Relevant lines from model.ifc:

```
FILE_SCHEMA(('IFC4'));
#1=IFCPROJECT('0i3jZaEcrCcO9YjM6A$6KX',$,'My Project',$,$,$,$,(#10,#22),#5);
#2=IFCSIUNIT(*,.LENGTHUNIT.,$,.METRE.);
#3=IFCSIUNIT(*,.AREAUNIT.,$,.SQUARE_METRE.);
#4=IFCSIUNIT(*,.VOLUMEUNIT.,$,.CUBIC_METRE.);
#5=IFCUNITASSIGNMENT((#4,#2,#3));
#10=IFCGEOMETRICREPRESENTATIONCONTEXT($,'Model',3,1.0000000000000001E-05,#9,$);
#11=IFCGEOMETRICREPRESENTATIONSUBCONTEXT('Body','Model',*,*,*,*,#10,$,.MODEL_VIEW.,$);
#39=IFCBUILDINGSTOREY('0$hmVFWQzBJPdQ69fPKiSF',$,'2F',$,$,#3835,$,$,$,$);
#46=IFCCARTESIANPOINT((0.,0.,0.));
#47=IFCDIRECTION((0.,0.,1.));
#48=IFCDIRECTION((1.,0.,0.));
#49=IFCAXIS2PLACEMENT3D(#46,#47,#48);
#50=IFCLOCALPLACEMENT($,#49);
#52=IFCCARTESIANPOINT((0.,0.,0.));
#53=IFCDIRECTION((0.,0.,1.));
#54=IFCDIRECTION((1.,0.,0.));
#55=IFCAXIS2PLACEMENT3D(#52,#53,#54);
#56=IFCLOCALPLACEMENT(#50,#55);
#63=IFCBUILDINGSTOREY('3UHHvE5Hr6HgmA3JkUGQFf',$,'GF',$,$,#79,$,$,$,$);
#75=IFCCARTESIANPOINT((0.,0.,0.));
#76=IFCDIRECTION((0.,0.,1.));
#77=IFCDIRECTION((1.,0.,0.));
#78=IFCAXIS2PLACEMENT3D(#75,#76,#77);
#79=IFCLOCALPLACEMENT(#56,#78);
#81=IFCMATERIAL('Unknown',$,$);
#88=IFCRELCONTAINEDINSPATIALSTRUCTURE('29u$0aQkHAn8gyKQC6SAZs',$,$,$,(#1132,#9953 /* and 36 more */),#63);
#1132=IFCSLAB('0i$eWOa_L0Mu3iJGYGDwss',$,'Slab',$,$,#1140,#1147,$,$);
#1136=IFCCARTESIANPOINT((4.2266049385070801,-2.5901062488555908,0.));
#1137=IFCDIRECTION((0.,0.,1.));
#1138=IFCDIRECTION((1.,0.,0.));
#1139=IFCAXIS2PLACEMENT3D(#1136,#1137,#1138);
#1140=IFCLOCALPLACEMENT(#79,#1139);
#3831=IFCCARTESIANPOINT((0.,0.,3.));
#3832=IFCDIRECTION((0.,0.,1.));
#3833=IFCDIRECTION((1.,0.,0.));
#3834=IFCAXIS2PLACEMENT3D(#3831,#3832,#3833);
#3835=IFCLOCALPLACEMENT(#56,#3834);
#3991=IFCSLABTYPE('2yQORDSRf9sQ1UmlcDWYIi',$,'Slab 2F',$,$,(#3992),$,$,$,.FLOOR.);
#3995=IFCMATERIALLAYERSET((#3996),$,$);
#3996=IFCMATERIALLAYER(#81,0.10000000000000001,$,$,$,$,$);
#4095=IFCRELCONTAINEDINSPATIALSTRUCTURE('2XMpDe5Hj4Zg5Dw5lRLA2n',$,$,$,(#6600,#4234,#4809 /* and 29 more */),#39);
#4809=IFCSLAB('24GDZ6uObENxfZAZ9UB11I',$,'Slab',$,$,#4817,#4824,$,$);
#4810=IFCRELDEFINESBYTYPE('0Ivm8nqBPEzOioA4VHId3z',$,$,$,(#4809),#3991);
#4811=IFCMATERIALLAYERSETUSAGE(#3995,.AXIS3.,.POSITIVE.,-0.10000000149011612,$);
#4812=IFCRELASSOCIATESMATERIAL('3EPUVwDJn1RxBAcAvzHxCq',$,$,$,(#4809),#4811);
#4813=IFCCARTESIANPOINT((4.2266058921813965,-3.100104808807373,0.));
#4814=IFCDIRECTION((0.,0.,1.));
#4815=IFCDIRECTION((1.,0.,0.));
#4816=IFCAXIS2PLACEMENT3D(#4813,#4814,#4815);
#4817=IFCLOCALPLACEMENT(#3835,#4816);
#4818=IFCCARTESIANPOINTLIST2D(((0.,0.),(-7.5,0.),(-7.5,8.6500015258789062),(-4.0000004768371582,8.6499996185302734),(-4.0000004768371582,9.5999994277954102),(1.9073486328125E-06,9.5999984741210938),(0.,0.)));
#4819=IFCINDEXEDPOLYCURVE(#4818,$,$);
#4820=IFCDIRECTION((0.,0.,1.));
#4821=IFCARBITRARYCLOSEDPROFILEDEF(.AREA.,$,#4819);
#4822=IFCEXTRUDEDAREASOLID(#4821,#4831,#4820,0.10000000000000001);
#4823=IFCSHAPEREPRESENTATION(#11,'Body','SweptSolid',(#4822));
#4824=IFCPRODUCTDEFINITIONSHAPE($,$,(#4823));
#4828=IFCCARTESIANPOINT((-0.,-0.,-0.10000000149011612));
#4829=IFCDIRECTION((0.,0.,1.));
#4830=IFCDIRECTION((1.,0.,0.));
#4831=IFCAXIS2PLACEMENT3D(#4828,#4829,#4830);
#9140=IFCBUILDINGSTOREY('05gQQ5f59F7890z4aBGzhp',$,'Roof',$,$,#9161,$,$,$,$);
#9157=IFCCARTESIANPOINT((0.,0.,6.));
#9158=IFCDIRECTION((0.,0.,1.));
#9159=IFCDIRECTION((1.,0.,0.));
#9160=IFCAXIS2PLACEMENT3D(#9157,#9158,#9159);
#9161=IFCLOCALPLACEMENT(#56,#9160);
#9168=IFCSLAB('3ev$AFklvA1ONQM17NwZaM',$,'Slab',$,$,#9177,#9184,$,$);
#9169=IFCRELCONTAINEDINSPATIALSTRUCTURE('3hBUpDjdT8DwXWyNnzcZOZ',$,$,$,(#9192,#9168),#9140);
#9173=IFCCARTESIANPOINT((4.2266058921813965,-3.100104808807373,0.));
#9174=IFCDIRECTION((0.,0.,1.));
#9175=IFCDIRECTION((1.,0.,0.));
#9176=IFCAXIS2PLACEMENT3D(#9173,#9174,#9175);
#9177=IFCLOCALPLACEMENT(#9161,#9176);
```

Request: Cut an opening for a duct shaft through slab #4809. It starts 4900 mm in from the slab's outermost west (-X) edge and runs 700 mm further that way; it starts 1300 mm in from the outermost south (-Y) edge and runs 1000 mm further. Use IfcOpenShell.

```python
import numpy as np
import ifcopenshell
import ifcopenshell.api.feature
import ifcopenshell.api.geometry
import ifcopenshell.api.root
import ifcopenshell.geom
import ifcopenshell.util.placement
import ifcopenshell.util.representation
import ifcopenshell.util.shape
import ifcopenshell.util.unit

model = ifcopenshell.open("model.ifc")
unit_scale = ifcopenshell.util.unit.calculate_unit_scale(model)
settings = ifcopenshell.geom.settings()


def volume(element):
    """Net volume in cubic metres, openings subtracted."""
    shape = ifcopenshell.geom.create_shape(settings, element)
    return ifcopenshell.util.shape.get_volume(shape.geometry)


slab = model.by_guid("24GDZ6uObENxfZAZ9UB11I")
before = volume(slab)

# Extent in the slab's own axes, in metres. The edges named are its -X and -Y sides.
slab_shape = ifcopenshell.geom.create_shape(settings, slab)
vertices = ifcopenshell.util.shape.get_vertices(slab_shape.geometry)
x_min, y_min, bottom = vertices.min(axis=0)
top = vertices[:, 2].max()

opening = ifcopenshell.api.root.create_entity(model, ifc_class="IfcOpeningElement", name="Duct shaft opening", predefined_type="OPENING")
context = ifcopenshell.util.representation.get_context(model, "Model", "Body", "MODEL_VIEW")
width, depth = 0.7, 1
outline = [(0.0, 0.0), (width, 0.0), (width, depth), (0.0, depth), (0.0, 0.0)]
# Overshoot both faces by 50 mm so the cut is clean.
shape = ifcopenshell.api.geometry.add_slab_representation(
    model, context=context, depth=top - bottom + 0.1, polyline=outline
)
ifcopenshell.api.geometry.assign_representation(model, product=opening, representation=shape)

matrix = ifcopenshell.util.placement.get_local_placement(slab.ObjectPlacement)
matrix[:, 3] = matrix @ np.append(np.array([x_min + 4.9, y_min + 1.3, bottom - 0.05]) / unit_scale, 1.0)
ifcopenshell.api.geometry.edit_object_placement(model, product=opening, matrix=matrix, is_si=False)
ifcopenshell.api.feature.add_feature(model, feature=opening, element=slab)

after = volume(slab)

print(f"slab volume {before:.3f} -> {after:.3f} m3")

model.write("model_v2.ifc")
```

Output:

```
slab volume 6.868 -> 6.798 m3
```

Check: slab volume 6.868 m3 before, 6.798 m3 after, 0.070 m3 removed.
